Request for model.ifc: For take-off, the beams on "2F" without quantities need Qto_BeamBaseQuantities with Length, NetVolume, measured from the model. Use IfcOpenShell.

First a look at what the model holds.

```python
import ifcopenshell
import ifcopenshell.util.element
import ifcopenshell.util.unit

model = ifcopenshell.open("model.ifc")
print(model.schema)
for unit_type in ("LENGTHUNIT", "AREAUNIT", "VOLUMEUNIT"):
    print(unit_type, ifcopenshell.util.unit.calculate_unit_scale(model, unit_type))
storey = next(s for s in model.by_type("IfcBuildingStorey") if s.Name == "2F")
beams = [e for e in ifcopenshell.util.element.get_decomposition(storey) if e.is_a("IfcBeam")]
for e in sorted(beams, key=lambda e: e.id()):
    print(e.id(), e.is_a(), e.Name, list(ifcopenshell.util.element.get_psets(e, qtos_only=True)), sep=" | ")
```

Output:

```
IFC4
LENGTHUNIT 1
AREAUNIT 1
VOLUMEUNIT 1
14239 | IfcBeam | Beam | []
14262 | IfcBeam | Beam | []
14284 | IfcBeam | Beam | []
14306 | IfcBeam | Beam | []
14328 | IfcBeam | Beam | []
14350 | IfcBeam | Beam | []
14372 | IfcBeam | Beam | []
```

```python
import ifcopenshell
import ifcopenshell.api.pset
import ifcopenshell.geom
import ifcopenshell.util.element
import ifcopenshell.util.shape
import ifcopenshell.util.unit

model = ifcopenshell.open("model.ifc")
unit_scale = ifcopenshell.util.unit.calculate_unit_scale(model)
volume_scale = ifcopenshell.util.unit.calculate_unit_scale(model, "VOLUMEUNIT")
settings = ifcopenshell.geom.settings()

storey = next(s for s in model.by_type("IfcBuildingStorey") if s.Name == "2F")
beams = [e for e in ifcopenshell.util.element.get_decomposition(storey) if e.is_a("IfcBeam")]

for e in sorted(beams, key=lambda e: e.id()):
    if ifcopenshell.util.element.get_psets(e, qtos_only=True, should_inherit=False):
        continue
    # Geometry comes back in metres, in the element's own axes.
    shape = ifcopenshell.geom.create_shape(settings, e)
    values = {
        "Length": ifcopenshell.util.shape.get_max_xyz(shape.geometry) / unit_scale,
        "NetVolume": ifcopenshell.util.shape.get_volume(shape.geometry) / volume_scale,
    }
    qto = ifcopenshell.api.pset.add_qto(model, product=e, name="Qto_BeamBaseQuantities")
    ifcopenshell.api.pset.edit_qto(model, qto=qto, properties=values)
    print(e.id(), {k: round(v, 3) for k, v in values.items()})

model.write("model_edited.ifc")
```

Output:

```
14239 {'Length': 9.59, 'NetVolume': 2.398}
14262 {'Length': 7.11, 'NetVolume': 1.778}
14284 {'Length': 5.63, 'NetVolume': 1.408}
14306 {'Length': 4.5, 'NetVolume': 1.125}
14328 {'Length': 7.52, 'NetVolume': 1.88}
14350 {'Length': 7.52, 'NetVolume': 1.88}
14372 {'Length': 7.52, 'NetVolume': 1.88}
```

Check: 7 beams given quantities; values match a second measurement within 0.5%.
